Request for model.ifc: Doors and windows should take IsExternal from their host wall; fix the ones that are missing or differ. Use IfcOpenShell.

First a look at what the model holds.

```python
import ifcopenshell
import ifcopenshell.util.element

model = ifcopenshell.open("model.ifc")
print(model.schema)
seen = {}
for e in model.by_type("IfcDoor") + model.by_type("IfcWindow"):
    if not e.FillsVoids:
        continue
    host = e.FillsVoids[0].RelatingOpeningElement.VoidsElements[0].RelatingBuildingElement
    own = ifcopenshell.util.element.get_pset(e, f"Pset_{e.is_a()[3:].removesuffix('StandardCase')}Common", "IsExternal")
    wall = ifcopenshell.util.element.get_pset(host, "Pset_WallCommon", "IsExternal")
    seen[e.is_a(), own, wall] = seen.get((e.is_a(), own, wall), 0) + 1
for (cls, own, wall), count in sorted(seen.items(), key=str):
    print(count, cls, "IsExternal:", own, "| host wall:", wall)
```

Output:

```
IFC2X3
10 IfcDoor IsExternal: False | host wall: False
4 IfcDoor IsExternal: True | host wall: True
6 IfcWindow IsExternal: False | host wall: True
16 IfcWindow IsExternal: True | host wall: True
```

```python
import ifcopenshell
import ifcopenshell.api.pset
import ifcopenshell.util.element

model = ifcopenshell.open("model.ifc")

count = 0
for ifc_class, pset_name in (("IfcDoor", "Pset_DoorCommon"), ("IfcWindow", "Pset_WindowCommon")):
    for e in model.by_type(ifc_class):
        if not e.FillsVoids:
            continue
        host = e.FillsVoids[0].RelatingOpeningElement.VoidsElements[0].RelatingBuildingElement
        external = ifcopenshell.util.element.get_pset(host, "Pset_WallCommon", "IsExternal")
        if external is None or ifcopenshell.util.element.get_pset(e, pset_name, "IsExternal") == external:
            continue
        pset = ifcopenshell.api.pset.add_pset(model, product=e, name=pset_name)
        ifcopenshell.api.pset.edit_pset(model, pset=pset, properties={"IsExternal": external})
        count += 1

print(count, "updated")

model.write("model_edited.ifc")
```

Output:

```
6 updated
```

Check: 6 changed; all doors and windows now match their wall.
